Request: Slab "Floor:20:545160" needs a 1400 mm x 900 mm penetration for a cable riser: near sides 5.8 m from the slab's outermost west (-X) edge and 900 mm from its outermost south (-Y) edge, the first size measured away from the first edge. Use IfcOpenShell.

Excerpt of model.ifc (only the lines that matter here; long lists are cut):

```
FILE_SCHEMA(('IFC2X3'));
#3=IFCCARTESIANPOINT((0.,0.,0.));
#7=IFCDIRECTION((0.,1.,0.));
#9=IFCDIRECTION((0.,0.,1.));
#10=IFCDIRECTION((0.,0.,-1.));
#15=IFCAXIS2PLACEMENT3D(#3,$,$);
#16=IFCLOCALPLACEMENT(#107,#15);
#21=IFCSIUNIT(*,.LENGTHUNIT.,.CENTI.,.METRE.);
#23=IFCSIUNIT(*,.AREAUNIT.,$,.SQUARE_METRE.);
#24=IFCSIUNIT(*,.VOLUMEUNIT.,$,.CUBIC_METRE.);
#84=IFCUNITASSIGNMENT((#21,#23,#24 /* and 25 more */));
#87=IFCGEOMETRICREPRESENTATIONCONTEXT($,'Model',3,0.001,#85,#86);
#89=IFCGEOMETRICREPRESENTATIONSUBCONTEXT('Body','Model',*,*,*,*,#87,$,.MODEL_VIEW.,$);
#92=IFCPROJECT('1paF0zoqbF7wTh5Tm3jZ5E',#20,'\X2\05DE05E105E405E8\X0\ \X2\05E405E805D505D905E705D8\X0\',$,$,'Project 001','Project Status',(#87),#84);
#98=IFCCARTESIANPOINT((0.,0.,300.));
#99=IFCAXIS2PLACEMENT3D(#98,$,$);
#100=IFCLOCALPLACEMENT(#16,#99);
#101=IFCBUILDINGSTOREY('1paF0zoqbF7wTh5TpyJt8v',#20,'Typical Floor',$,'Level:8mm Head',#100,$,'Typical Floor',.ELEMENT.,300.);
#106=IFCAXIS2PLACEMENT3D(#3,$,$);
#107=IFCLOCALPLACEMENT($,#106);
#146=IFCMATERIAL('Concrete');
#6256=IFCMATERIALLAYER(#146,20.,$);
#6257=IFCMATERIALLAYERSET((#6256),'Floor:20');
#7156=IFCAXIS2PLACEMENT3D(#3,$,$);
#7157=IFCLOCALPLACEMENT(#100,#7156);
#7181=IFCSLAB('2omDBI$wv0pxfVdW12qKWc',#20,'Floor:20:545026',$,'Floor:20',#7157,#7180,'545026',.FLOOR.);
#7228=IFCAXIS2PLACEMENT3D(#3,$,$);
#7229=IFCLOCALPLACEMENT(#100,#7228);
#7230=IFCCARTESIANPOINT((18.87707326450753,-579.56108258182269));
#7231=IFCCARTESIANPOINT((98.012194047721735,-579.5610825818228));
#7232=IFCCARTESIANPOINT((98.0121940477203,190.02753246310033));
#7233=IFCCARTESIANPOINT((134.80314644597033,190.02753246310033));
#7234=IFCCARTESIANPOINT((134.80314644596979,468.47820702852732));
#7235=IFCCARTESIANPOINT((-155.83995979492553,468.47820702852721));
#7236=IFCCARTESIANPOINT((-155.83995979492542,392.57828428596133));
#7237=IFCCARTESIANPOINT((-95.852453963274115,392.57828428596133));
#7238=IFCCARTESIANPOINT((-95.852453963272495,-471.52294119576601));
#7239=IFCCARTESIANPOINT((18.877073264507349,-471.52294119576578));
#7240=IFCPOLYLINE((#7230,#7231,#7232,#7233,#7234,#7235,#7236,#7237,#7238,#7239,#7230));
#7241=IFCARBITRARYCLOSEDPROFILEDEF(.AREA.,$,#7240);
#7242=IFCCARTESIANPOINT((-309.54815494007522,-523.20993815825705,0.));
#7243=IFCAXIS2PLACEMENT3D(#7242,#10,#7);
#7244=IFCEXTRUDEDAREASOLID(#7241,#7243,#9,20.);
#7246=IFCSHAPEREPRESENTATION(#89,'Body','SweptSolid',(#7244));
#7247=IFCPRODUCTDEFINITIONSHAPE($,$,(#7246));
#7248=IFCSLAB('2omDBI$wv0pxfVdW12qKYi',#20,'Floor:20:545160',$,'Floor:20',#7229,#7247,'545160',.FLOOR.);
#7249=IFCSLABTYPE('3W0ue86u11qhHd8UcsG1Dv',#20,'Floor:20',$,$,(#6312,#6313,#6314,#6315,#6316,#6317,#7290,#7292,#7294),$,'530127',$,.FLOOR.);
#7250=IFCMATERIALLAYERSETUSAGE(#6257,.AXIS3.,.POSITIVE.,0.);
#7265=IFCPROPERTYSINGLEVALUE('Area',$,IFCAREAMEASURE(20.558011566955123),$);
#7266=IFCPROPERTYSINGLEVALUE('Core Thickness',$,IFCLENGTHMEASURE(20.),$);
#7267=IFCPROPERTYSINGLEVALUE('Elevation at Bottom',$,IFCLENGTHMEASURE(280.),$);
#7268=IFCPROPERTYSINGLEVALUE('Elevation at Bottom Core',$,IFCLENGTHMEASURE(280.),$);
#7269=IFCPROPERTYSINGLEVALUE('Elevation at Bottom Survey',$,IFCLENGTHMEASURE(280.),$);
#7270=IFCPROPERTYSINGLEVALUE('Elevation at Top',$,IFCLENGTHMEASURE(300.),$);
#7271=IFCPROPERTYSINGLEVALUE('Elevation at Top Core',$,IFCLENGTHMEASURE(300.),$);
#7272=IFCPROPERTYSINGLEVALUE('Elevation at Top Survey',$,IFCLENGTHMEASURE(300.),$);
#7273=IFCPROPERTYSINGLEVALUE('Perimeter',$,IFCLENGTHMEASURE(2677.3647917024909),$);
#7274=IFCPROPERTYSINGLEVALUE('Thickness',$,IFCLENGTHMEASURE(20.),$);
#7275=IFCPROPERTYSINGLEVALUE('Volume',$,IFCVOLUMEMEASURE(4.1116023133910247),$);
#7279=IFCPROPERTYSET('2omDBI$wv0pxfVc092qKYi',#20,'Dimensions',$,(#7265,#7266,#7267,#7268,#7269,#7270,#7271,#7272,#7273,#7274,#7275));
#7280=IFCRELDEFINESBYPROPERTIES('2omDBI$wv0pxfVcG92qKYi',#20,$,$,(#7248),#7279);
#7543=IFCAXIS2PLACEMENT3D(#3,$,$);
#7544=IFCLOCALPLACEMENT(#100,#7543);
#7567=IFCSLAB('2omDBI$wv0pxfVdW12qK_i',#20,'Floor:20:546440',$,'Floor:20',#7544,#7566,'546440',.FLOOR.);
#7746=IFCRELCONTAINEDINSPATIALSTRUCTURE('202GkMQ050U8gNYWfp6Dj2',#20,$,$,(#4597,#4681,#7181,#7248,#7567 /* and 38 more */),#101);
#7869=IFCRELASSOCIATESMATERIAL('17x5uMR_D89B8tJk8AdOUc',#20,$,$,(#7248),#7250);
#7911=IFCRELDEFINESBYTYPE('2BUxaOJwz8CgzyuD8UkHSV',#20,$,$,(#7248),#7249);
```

```python
import numpy as np
import ifcopenshell
import ifcopenshell.api.feature
import ifcopenshell.api.geometry
import ifcopenshell.api.pset
import ifcopenshell.api.root
import ifcopenshell.geom
import ifcopenshell.util.element
import ifcopenshell.util.placement
import ifcopenshell.util.representation
import ifcopenshell.util.shape
import ifcopenshell.util.unit

model = ifcopenshell.open("model.ifc")
unit_scale = ifcopenshell.util.unit.calculate_unit_scale(model)
area_scale = ifcopenshell.util.unit.calculate_unit_scale(model, "AREAUNIT")
volume_scale = ifcopenshell.util.unit.calculate_unit_scale(model, "VOLUMEUNIT")
settings = ifcopenshell.geom.settings()


def volume(element):
    """Net volume in cubic metres, openings subtracted."""
    shape = ifcopenshell.geom.create_shape(settings, element)
    return ifcopenshell.util.shape.get_volume(shape.geometry)


slab = model.by_guid("2omDBI$wv0pxfVdW12qKYi")
before = volume(slab)

# Extent in the slab's own axes, in metres. The edges named are its -X and -Y sides.
slab_shape = ifcopenshell.geom.create_shape(settings, slab)
vertices = ifcopenshell.util.shape.get_vertices(slab_shape.geometry)
x_min, y_min, bottom = vertices.min(axis=0)
top = vertices[:, 2].max()

opening = ifcopenshell.api.root.create_entity(model, ifc_class="IfcOpeningElement", name="Cable riser opening")
context = ifcopenshell.util.representation.get_context(model, "Model", "Body", "MODEL_VIEW")
width, depth = 1.4, 0.9
outline = [(0.0, 0.0), (width, 0.0), (width, depth), (0.0, depth), (0.0, 0.0)]
# Overshoot both faces by 50 mm so the cut is clean.
shape = ifcopenshell.api.geometry.add_slab_representation(
    model, context=context, depth=top - bottom + 0.1, polyline=outline
)
ifcopenshell.api.geometry.assign_representation(model, product=opening, representation=shape)

matrix = ifcopenshell.util.placement.get_local_placement(slab.ObjectPlacement)
matrix[:, 3] = matrix @ np.append(np.array([x_min + 5.8, y_min + 0.9, bottom - 0.05]) / unit_scale, 1.0)
ifcopenshell.api.geometry.edit_object_placement(model, product=opening, matrix=matrix, is_si=False)
ifcopenshell.api.feature.add_feature(model, feature=opening, element=slab)

after = volume(slab)

# Update the slab's stored quantities.
pset = model.by_id(ifcopenshell.util.element.get_pset(slab, "Dimensions", should_inherit=False)["id"])
ifcopenshell.api.pset.edit_pset(model, pset=pset, properties={
    "Area": model.create_entity("IfcAreaMeasure", after / (top - bottom) / area_scale),
    "Volume": model.create_entity("IfcVolumeMeasure", after / volume_scale),
})

print(f"slab volume {before:.3f} -> {after:.3f} m3")

model.write("model_edited.ifc")
```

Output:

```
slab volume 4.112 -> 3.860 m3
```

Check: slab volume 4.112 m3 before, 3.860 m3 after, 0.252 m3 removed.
